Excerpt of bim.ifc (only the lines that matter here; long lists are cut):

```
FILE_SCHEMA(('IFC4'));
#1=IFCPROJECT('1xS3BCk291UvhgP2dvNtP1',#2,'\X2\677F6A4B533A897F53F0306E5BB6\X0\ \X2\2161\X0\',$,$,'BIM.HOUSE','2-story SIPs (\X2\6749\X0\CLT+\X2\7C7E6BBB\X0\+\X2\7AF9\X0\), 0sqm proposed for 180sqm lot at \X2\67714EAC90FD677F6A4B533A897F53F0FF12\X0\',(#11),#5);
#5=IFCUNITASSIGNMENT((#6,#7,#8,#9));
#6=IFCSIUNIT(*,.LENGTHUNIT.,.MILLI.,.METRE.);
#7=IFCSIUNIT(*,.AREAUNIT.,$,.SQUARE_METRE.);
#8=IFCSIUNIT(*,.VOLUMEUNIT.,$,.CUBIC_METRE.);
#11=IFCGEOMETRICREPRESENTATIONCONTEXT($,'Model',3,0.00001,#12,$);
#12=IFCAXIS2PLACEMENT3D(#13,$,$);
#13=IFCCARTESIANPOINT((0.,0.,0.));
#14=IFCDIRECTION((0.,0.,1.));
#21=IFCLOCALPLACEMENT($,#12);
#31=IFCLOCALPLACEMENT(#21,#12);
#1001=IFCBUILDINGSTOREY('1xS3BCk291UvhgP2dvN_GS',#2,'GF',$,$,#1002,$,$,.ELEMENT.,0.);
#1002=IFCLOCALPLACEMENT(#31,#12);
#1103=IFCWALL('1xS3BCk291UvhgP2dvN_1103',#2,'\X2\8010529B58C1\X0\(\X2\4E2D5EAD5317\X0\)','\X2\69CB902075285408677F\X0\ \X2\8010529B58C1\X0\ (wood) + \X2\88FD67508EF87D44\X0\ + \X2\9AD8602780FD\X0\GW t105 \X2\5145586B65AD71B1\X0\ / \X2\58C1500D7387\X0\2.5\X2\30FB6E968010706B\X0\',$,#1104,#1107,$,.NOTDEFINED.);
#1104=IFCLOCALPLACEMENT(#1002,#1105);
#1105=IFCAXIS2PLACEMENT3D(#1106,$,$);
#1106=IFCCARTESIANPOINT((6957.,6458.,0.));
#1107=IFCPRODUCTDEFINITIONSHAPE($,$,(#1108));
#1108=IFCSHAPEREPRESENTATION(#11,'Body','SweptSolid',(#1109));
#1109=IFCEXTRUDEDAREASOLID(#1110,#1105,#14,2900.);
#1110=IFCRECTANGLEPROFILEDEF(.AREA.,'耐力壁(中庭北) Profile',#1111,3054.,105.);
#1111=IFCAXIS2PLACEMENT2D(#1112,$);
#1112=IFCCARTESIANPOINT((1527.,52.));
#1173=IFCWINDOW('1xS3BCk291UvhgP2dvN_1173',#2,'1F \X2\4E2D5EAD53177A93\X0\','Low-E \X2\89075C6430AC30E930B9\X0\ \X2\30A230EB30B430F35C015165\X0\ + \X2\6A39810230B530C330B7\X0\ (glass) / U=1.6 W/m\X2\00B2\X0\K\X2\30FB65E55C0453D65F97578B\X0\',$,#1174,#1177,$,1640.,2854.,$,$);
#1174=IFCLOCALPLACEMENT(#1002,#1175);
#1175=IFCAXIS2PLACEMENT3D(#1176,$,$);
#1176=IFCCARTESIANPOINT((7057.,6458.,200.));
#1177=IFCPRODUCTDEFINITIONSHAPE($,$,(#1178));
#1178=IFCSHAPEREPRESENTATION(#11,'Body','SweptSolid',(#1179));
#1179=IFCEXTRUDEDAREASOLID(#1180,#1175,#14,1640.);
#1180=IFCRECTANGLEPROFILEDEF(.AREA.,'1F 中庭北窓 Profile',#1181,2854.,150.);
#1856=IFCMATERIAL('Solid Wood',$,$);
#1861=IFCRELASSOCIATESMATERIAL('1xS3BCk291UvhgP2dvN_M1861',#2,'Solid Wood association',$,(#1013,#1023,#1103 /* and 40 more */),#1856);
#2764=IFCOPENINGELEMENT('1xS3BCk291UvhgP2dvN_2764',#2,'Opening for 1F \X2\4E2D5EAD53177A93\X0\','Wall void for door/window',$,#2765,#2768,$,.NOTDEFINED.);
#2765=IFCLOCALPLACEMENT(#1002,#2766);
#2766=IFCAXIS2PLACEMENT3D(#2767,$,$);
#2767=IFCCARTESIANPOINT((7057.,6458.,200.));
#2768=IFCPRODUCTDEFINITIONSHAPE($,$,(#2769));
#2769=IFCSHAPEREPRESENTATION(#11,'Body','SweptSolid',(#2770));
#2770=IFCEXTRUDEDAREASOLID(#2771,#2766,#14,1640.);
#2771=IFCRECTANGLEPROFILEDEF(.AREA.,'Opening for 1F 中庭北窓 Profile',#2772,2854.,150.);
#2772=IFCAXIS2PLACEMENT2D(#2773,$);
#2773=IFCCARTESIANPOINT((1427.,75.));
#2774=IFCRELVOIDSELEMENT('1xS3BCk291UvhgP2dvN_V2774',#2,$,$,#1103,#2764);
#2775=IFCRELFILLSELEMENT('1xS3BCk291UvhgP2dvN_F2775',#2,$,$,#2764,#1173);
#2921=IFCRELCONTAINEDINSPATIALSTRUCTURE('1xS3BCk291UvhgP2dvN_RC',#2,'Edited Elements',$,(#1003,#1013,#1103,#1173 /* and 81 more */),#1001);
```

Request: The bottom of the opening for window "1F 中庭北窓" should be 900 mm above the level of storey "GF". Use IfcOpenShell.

```python
import numpy as np
import ifcopenshell
import ifcopenshell.api.geometry
import ifcopenshell.geom
import ifcopenshell.util.element
import ifcopenshell.util.placement
import ifcopenshell.util.shape
import ifcopenshell.util.unit

model = ifcopenshell.open("bim.ifc")
unit_scale = ifcopenshell.util.unit.calculate_unit_scale(model)

window = model.by_guid("1xS3BCk291UvhgP2dvN_1173")
opening = window.FillsVoids[0].RelatingOpeningElement
storey = ifcopenshell.util.element.get_container(window, ifc_class="IfcBuildingStorey")
level = ifcopenshell.util.placement.get_local_placement(storey.ObjectPlacement)[2, 3]

# The opening's origin need not be at the sill, so measure its lowest point.
shape = ifcopenshell.geom.create_shape(ifcopenshell.geom.settings(), opening)
bottom = ifcopenshell.util.shape.get_shape_bottom_elevation(shape, shape.geometry) / unit_scale
dz = level + 0.9 / unit_scale - bottom

shift = np.array([0.0, 0.0, dz])
# The window is not placed relative to its opening, so move both.
for product in (opening, window):
    matrix = ifcopenshell.util.placement.get_local_placement(product.ObjectPlacement)
    matrix[:3, 3] += shift
    ifcopenshell.api.geometry.edit_object_placement(model, product=product, matrix=matrix, is_si=False)

print(f"moved by {dz * unit_scale:+.3f} m")

model.write("bim_updated.ifc")
```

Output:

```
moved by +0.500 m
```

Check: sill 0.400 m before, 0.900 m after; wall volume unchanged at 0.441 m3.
